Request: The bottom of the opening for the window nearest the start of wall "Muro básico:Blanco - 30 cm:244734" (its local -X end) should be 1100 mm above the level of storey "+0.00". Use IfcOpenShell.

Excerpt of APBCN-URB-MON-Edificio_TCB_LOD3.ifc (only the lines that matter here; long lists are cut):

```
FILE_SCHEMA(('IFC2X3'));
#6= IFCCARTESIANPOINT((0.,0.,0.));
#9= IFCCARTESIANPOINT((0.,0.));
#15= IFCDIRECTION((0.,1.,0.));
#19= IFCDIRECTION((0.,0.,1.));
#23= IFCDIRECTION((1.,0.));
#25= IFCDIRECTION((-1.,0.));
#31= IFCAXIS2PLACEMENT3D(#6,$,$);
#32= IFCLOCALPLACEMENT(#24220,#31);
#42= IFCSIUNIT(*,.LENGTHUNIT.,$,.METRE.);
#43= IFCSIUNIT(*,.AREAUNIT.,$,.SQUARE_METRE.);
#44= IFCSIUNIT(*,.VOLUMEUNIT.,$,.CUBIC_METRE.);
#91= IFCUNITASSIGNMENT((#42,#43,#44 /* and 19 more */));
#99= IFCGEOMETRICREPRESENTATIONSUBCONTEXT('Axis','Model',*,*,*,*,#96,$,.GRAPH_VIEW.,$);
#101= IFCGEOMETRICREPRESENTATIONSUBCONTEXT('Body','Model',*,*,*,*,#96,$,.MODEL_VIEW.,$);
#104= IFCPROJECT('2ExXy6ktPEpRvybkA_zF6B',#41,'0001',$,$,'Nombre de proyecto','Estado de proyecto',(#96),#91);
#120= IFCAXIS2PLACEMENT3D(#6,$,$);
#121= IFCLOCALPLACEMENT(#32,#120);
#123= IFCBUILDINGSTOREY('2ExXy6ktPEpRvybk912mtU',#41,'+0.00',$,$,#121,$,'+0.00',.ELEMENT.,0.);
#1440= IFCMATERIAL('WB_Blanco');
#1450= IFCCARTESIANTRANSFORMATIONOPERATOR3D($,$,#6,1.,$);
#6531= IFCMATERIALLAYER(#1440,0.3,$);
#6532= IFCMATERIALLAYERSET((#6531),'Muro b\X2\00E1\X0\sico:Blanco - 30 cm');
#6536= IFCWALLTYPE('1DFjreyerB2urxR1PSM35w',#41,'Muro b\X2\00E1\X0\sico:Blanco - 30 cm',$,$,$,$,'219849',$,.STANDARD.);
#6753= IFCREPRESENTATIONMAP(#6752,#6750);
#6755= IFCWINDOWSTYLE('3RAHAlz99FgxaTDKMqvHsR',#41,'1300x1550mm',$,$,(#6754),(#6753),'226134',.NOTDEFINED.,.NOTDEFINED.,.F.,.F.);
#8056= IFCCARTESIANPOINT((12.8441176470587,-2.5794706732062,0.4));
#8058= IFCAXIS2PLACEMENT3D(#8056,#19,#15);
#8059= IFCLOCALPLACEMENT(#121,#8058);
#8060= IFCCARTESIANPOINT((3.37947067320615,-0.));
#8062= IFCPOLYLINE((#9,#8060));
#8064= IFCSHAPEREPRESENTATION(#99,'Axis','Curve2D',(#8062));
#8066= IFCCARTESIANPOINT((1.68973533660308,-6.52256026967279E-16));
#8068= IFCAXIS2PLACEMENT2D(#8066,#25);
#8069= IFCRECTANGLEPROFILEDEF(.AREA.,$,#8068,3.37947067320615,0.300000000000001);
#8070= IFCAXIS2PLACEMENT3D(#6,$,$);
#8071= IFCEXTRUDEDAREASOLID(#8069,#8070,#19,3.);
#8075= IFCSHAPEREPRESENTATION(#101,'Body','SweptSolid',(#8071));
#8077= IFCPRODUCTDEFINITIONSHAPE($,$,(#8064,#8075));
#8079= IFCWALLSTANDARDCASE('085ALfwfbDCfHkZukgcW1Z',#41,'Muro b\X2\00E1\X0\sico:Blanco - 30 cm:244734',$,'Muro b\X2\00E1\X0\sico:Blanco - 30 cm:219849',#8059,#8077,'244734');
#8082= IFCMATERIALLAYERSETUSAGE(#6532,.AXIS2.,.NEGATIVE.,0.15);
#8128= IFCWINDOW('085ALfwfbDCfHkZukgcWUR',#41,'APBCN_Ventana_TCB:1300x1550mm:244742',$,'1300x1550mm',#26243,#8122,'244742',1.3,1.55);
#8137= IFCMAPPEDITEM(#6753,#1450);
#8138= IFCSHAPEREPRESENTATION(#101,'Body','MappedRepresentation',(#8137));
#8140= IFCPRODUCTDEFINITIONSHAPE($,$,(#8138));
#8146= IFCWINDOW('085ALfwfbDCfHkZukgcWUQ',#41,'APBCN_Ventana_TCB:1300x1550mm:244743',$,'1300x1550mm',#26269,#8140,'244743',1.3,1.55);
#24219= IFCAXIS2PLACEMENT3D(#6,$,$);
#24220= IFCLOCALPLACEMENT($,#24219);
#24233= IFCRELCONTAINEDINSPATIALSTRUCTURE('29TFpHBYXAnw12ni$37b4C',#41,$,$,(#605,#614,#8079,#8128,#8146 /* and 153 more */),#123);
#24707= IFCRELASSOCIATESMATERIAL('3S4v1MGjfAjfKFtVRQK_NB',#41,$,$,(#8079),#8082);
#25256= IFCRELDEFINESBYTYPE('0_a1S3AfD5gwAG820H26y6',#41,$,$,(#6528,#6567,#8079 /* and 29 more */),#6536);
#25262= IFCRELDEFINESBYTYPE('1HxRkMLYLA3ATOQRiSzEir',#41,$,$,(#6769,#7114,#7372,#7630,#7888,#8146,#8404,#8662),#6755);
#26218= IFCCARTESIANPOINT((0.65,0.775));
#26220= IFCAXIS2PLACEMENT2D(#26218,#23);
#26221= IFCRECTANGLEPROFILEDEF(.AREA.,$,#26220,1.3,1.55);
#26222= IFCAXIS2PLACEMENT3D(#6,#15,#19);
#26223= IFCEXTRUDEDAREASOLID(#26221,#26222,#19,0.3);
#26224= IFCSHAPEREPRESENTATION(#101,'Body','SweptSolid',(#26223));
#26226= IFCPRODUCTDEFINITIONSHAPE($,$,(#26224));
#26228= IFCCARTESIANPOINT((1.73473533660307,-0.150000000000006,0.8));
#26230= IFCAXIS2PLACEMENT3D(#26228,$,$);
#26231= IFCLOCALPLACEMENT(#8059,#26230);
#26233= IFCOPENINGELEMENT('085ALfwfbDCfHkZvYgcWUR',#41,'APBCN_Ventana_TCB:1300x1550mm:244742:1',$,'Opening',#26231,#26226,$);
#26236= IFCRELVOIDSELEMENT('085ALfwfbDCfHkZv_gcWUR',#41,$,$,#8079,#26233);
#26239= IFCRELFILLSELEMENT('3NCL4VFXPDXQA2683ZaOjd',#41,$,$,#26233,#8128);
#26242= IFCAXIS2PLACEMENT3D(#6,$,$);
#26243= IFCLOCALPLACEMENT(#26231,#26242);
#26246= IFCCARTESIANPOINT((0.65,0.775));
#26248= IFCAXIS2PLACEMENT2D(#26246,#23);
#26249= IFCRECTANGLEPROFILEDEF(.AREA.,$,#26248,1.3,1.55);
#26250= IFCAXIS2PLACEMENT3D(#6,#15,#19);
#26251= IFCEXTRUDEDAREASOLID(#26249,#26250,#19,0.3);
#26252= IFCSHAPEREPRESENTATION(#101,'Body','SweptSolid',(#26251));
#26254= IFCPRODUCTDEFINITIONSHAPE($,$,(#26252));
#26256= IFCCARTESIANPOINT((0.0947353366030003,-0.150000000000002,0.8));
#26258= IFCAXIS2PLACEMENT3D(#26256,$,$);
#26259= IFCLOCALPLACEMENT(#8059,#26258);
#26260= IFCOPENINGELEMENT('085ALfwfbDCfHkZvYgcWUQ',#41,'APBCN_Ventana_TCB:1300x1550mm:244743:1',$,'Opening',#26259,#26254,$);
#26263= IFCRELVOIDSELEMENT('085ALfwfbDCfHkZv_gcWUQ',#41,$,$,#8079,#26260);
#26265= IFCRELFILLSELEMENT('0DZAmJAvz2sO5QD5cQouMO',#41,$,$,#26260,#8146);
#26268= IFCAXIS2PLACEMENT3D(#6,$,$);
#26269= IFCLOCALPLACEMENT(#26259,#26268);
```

```python
import numpy as np
import ifcopenshell
import ifcopenshell.api.geometry
import ifcopenshell.geom
import ifcopenshell.util.element
import ifcopenshell.util.placement
import ifcopenshell.util.shape
import ifcopenshell.util.unit

model = ifcopenshell.open("APBCN-URB-MON-Edificio_TCB_LOD3.ifc")
unit_scale = ifcopenshell.util.unit.calculate_unit_scale(model)

window = model.by_id(8146)
opening = window.FillsVoids[0].RelatingOpeningElement
storey = ifcopenshell.util.element.get_container(window, ifc_class="IfcBuildingStorey")
level = ifcopenshell.util.placement.get_local_placement(storey.ObjectPlacement)[2, 3]

# The opening's origin need not be at the sill, so measure its lowest point.
shape = ifcopenshell.geom.create_shape(ifcopenshell.geom.settings(), opening)
bottom = ifcopenshell.util.shape.get_shape_bottom_elevation(shape, shape.geometry) / unit_scale
dz = level + 1.1 / unit_scale - bottom

shift = np.array([0.0, 0.0, dz])
# The window is placed relative to its opening, so it follows when the opening moves.
matrix = ifcopenshell.util.placement.get_local_placement(opening.ObjectPlacement)
matrix[:3, 3] += shift
ifcopenshell.api.geometry.edit_object_placement(
    model, product=opening, matrix=matrix, is_si=False, should_transform_children=True
)

print(f"moved by {dz * unit_scale:+.3f} m")

model.write("APBCN-URB-MON-Edificio_TCB_LOD3_v2.ifc")
```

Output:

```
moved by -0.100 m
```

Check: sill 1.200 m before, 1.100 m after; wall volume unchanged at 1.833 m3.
